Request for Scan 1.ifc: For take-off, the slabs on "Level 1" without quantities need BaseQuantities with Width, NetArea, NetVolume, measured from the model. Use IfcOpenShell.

First a look at what the model holds.

```python
import ifcopenshell
import ifcopenshell.util.element
import ifcopenshell.util.unit

model = ifcopenshell.open("Scan 1.ifc")
print(model.schema)
for unit_type in ("LENGTHUNIT", "AREAUNIT", "VOLUMEUNIT"):
    print(unit_type, ifcopenshell.util.unit.calculate_unit_scale(model, unit_type))
storey = next(s for s in model.by_type("IfcBuildingStorey") if s.Name == "Level 1")
slabs = [e for e in ifcopenshell.util.element.get_decomposition(storey) if e.is_a("IfcSlab")]
for e in sorted(slabs, key=lambda e: e.id()):
    print(e.id(), e.is_a(), e.Name, list(ifcopenshell.util.element.get_psets(e, qtos_only=True)), sep=" | ")
```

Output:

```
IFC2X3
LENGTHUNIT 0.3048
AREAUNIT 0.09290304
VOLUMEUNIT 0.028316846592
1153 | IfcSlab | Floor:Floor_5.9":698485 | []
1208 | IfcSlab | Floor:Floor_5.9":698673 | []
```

```python
import ifcopenshell
import ifcopenshell.api.pset
import ifcopenshell.geom
import ifcopenshell.util.element
import ifcopenshell.util.shape
import ifcopenshell.util.unit

model = ifcopenshell.open("Scan 1.ifc")
unit_scale = ifcopenshell.util.unit.calculate_unit_scale(model)
area_scale = ifcopenshell.util.unit.calculate_unit_scale(model, "AREAUNIT")
volume_scale = ifcopenshell.util.unit.calculate_unit_scale(model, "VOLUMEUNIT")
settings = ifcopenshell.geom.settings()

storey = next(s for s in model.by_type("IfcBuildingStorey") if s.Name == "Level 1")
slabs = [e for e in ifcopenshell.util.element.get_decomposition(storey) if e.is_a("IfcSlab")]

for e in sorted(slabs, key=lambda e: e.id()):
    if ifcopenshell.util.element.get_psets(e, qtos_only=True, should_inherit=False):
        continue
    # Geometry comes back in metres, in the element's own axes.
    shape = ifcopenshell.geom.create_shape(settings, e)
    values = {
        "Width": ifcopenshell.util.shape.get_z(shape.geometry) / unit_scale,
        "NetArea": ifcopenshell.util.shape.get_footprint_area(shape.geometry) / area_scale,
        "NetVolume": ifcopenshell.util.shape.get_volume(shape.geometry) / volume_scale,
    }
    qto = ifcopenshell.api.pset.add_qto(model, product=e, name="BaseQuantities")
    ifcopenshell.api.pset.edit_qto(model, qto=qto, properties=values)
    print(e.id(), {k: round(v, 3) for k, v in values.items()})

model.write("Scan 1_edited.ifc")
```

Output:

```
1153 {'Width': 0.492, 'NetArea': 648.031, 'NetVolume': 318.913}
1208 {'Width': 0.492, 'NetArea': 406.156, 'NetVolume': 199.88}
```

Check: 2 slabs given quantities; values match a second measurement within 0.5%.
